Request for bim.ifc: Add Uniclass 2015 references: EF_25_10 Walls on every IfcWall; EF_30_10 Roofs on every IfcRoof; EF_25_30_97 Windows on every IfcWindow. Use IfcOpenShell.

First a look at what the model holds.

```python
import ifcopenshell

model = ifcopenshell.open("bim.ifc")
print(model.schema)
print("classifications:", [c.Name for c in model.by_type("IfcClassification")])
for ifc_class in ("IfcDoor", "IfcRoof", "IfcStair", "IfcWall", "IfcWindow"):
    print(ifc_class, len(model.by_type(ifc_class)))
```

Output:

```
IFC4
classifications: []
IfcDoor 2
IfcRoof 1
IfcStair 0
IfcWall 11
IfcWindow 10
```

```python
import ifcopenshell
import ifcopenshell.api.classification

model = ifcopenshell.open("bim.ifc")

system = ifcopenshell.api.classification.add_classification(model, classification="Uniclass 2015")

codes = {
    "IfcWall": ("EF_25_10", "Walls"),
    "IfcRoof": ("EF_30_10", "Roofs"),
    "IfcWindow": ("EF_25_30_97", "Windows"),
}
for ifc_class, (code, name) in codes.items():
    products = model.by_type(ifc_class)
    ifcopenshell.api.classification.add_reference(
        model, products=products, classification=system, identification=code, name=name
    )
    print(code, len(products))

model.write("bim-out.ifc")
```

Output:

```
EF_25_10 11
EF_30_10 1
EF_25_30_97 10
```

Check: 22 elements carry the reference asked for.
